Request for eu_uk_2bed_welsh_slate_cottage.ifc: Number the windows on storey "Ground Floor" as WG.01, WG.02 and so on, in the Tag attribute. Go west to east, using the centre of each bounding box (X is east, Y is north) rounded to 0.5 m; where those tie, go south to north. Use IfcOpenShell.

First a look at what the model holds.

```python
import ifcopenshell
import ifcopenshell.util.element
import ifcopenshell.util.placement

model = ifcopenshell.open("eu_uk_2bed_welsh_slate_cottage.ifc")
print(model.schema)
storey = next(s for s in model.by_type("IfcBuildingStorey") if s.Name == "Ground Floor")
windows = [e for e in ifcopenshell.util.element.get_decomposition(storey) if e.is_a("IfcWindow")]
for e in sorted(windows, key=lambda e: e.id()):
    origin = ifcopenshell.util.placement.get_local_placement(e.ObjectPlacement)[:3, 3]
    print(e.id(), e.Tag, e.Name, origin.round(2) + 0.0, sep=" | ")
```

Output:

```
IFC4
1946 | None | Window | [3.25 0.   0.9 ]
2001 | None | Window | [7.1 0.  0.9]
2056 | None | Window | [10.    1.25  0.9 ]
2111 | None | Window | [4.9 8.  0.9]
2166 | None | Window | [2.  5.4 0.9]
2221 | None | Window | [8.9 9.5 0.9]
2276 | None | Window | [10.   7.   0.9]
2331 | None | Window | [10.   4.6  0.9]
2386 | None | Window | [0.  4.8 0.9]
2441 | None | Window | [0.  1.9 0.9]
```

```python
import ifcopenshell
import ifcopenshell.geom
import ifcopenshell.util.element
import ifcopenshell.util.shape

model = ifcopenshell.open("eu_uk_2bed_welsh_slate_cottage.ifc")
settings = ifcopenshell.geom.settings()
settings.set("use-world-coords", True)


def centre(element):
    shape = ifcopenshell.geom.create_shape(settings, element)
    return ifcopenshell.util.shape.get_bbox_centroid(shape.geometry)


storey = next(s for s in model.by_type("IfcBuildingStorey") if s.Name == "Ground Floor")
windows = [e for e in ifcopenshell.util.element.get_decomposition(storey) if e.is_a("IfcWindow")]

# Insertion points can sit at a corner or the storey origin, so sort by the geometry (in metres).
centres = {e: centre(e) for e in windows}
windows.sort(key=lambda e: (round(centres[e][0] / 0.5), centres[e][1]))

for i, e in enumerate(windows, start=1):
    number = f"WG.{i:02d}"
    e.Tag = number
    print(e.id(), number)

model.write("eu_uk_2bed_welsh_slate_cottage_edited.ifc")
```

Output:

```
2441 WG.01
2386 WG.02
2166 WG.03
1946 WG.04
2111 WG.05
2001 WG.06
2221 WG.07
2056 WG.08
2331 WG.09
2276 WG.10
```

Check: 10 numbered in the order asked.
